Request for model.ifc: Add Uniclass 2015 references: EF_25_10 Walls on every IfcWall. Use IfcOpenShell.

First a look at what the model holds.

```python
import ifcopenshell

model = ifcopenshell.open("model.ifc")
print(model.schema)
print("classifications:", [c.Name for c in model.by_type("IfcClassification")])
for ifc_class in ("IfcDoor", "IfcRoof", "IfcStair", "IfcWall", "IfcWindow"):
    print(ifc_class, len(model.by_type(ifc_class)))
```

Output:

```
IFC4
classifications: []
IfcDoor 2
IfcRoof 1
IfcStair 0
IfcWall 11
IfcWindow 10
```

```python
import ifcopenshell
import ifcopenshell.api.classification

model = ifcopenshell.open("model.ifc")

system = ifcopenshell.api.classification.add_classification(model, classification="Uniclass 2015")

codes = {
    "IfcWall": ("EF_25_10", "Walls"),
}
for ifc_class, (code, name) in codes.items():
    products = model.by_type(ifc_class)
    ifcopenshell.api.classification.add_reference(
        model, products=products, classification=system, identification=code, name=name
    )
    print(code, len(products))

model.write("model_v2.ifc")
```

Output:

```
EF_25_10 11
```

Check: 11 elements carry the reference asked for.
